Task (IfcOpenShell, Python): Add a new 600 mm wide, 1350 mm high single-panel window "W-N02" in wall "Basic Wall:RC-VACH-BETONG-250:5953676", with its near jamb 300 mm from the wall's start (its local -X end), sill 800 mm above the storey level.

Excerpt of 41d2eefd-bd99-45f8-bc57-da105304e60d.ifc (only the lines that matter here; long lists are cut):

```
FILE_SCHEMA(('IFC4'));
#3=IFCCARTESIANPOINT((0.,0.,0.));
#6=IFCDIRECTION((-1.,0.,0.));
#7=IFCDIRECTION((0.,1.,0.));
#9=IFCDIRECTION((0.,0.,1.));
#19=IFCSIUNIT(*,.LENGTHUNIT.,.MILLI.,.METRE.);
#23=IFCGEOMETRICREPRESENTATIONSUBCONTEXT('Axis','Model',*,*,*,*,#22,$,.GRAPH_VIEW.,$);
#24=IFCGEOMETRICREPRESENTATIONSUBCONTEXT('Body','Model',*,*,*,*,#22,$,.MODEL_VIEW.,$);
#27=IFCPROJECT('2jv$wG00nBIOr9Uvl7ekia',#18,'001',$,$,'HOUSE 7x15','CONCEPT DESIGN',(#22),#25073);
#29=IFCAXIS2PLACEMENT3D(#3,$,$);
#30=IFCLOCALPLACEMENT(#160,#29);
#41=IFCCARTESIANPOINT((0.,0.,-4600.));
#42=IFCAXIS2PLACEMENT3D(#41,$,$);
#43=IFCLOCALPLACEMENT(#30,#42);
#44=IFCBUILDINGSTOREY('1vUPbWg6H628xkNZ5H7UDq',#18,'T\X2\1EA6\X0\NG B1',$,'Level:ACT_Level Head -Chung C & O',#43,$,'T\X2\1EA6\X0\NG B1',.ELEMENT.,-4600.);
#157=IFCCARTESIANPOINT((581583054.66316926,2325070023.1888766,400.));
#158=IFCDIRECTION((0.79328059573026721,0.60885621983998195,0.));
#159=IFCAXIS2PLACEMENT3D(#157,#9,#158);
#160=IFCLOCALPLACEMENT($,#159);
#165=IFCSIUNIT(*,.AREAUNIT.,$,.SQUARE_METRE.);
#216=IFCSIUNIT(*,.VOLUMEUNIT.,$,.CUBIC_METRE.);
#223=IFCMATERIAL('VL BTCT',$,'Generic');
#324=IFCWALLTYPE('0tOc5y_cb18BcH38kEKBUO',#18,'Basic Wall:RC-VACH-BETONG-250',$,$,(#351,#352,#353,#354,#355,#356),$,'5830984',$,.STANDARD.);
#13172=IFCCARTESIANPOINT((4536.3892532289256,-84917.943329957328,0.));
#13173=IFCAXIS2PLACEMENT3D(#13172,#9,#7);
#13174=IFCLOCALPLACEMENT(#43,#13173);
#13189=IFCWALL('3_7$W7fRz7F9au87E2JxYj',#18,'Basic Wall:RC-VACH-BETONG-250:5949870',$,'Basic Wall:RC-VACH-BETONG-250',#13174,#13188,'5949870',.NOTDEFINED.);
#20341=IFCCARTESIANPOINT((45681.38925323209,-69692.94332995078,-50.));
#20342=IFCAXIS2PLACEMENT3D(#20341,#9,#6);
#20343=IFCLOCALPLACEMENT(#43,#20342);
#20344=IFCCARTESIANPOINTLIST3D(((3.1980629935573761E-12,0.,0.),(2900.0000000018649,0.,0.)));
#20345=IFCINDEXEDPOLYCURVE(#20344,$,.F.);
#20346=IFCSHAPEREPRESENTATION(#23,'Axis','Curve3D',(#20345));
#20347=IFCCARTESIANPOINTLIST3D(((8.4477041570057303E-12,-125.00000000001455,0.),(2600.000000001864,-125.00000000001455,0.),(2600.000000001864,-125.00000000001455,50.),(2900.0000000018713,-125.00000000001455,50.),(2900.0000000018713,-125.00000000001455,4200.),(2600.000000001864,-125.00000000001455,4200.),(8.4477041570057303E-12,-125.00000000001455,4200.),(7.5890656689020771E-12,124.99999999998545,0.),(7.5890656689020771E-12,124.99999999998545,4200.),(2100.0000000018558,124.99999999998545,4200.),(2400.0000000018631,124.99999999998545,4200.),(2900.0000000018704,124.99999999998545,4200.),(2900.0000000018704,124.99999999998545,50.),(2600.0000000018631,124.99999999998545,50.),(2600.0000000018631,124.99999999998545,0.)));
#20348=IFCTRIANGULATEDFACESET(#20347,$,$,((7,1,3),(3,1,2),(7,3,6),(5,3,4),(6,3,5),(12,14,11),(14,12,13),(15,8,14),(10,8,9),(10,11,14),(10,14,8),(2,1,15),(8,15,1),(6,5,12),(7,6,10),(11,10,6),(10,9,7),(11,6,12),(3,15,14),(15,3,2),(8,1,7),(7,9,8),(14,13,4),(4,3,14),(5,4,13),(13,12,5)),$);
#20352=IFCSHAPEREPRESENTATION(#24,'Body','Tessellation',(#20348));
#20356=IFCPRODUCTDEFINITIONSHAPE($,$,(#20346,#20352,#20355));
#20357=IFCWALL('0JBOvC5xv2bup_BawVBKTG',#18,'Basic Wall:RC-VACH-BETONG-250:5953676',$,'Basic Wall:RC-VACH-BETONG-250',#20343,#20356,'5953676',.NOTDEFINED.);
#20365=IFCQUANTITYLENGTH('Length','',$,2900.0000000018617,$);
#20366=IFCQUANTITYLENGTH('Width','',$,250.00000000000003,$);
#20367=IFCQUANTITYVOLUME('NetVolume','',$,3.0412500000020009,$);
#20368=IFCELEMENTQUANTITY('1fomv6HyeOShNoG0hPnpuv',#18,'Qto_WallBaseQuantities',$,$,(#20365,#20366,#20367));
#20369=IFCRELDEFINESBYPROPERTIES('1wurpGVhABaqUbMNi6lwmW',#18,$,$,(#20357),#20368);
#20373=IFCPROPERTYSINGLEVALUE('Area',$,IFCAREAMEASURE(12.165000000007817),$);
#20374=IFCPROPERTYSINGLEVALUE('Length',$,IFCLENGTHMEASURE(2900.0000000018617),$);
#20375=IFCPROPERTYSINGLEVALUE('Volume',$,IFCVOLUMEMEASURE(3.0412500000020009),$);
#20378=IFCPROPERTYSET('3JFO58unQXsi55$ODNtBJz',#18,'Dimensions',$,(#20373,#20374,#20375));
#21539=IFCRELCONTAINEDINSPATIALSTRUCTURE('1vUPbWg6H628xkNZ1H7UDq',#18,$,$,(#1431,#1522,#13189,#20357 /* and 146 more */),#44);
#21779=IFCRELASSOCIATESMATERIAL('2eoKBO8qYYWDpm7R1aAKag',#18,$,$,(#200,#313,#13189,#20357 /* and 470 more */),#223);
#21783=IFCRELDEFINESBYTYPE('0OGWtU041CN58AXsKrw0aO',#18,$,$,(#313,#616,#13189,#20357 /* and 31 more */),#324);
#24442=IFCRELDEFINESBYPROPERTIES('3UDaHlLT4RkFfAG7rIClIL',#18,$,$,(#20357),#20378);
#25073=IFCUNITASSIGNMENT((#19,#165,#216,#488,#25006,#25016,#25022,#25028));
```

```python
import numpy as np
import ifcopenshell
import ifcopenshell.api.feature
import ifcopenshell.api.geometry
import ifcopenshell.api.pset
import ifcopenshell.api.root
import ifcopenshell.api.spatial
import ifcopenshell.geom
import ifcopenshell.util.element
import ifcopenshell.util.placement
import ifcopenshell.util.representation
import ifcopenshell.util.shape
import ifcopenshell.util.unit

model = ifcopenshell.open("41d2eefd-bd99-45f8-bc57-da105304e60d.ifc")
unit_scale = ifcopenshell.util.unit.calculate_unit_scale(model)
area_scale = ifcopenshell.util.unit.calculate_unit_scale(model, "AREAUNIT")
volume_scale = ifcopenshell.util.unit.calculate_unit_scale(model, "VOLUMEUNIT")
settings = ifcopenshell.geom.settings()


def volume(element):
    """Net volume in cubic metres, openings subtracted."""
    shape = ifcopenshell.geom.create_shape(settings, element)
    return ifcopenshell.util.shape.get_volume(shape.geometry)


wall = model.by_guid("0JBOvC5xv2bup_BawVBKTG")
storey = ifcopenshell.util.element.get_container(wall, ifc_class="IfcBuildingStorey")
context = ifcopenshell.util.representation.get_context(model, "Model", "Body", "MODEL_VIEW")
before = volume(wall)

width, height, from_end, sill = 0.6, 1.35, 0.3, 0.8  # metres

# The wall runs along its own X axis, and the end named is its -X end.
wall_shape = ifcopenshell.geom.create_shape(settings, wall)
x, y, z = ifcopenshell.util.shape.get_vertices(wall_shape.geometry).T
start = x.min() + from_end
face, thickness = float(y.min()), float(y.max() - y.min())
wall_matrix = ifcopenshell.util.placement.get_local_placement(wall.ObjectPlacement)
level = ifcopenshell.util.placement.get_local_placement(storey.ObjectPlacement)[2, 3]


def in_wall(x, y):
    """Placement at x, y metres in the wall's axes, at sill height."""
    matrix = wall_matrix.copy()
    matrix[:, 3] = wall_matrix @ np.array([x / unit_scale, y / unit_scale, 0.0, 1.0])
    matrix[2, 3] = level + sill / unit_scale
    return matrix


# Opening: a box that overshoots both wall faces by 50 mm.
opening = ifcopenshell.api.root.create_entity(model, ifc_class="IfcOpeningElement", predefined_type="OPENING")
box = ifcopenshell.api.geometry.add_wall_representation(
    model, context=context, length=width, height=height, thickness=thickness + 0.1
)
ifcopenshell.api.geometry.assign_representation(model, product=opening, representation=box)
ifcopenshell.api.geometry.edit_object_placement(model, product=opening, matrix=in_wall(start, face - 0.05), is_si=False)
ifcopenshell.api.feature.add_feature(model, feature=opening, element=wall)

window = ifcopenshell.api.root.create_entity(model, ifc_class="IfcWindow", name="W-N02", predefined_type="WINDOW")
window.OverallWidth, window.OverallHeight = width / unit_scale, height / unit_scale
window.PartitioningType = "SINGLE_PANEL"
body = ifcopenshell.api.geometry.add_window_representation(
    model,
    context=context,
    overall_width=window.OverallWidth,
    overall_height=window.OverallHeight,
    partition_type="SINGLE_PANEL",
)
ifcopenshell.api.geometry.assign_representation(model, product=window, representation=body)
ifcopenshell.api.spatial.assign_container(model, products=[window], relating_structure=storey)
ifcopenshell.api.feature.add_filling(model, opening=opening, element=window)

# Centre the window in the wall's thickness.
ifcopenshell.api.geometry.edit_object_placement(model, product=window, matrix=in_wall(start, face), is_si=False)
window_shape = ifcopenshell.geom.create_shape(settings, window)
depth = ifcopenshell.util.shape.get_vertices(window_shape.geometry)[:, 1]
offset = face + thickness / 2 - (depth.min() + depth.max()) / 2
ifcopenshell.api.geometry.edit_object_placement(model, product=window, matrix=in_wall(start, offset), is_si=False)

after = volume(wall)

# Update the wall's stored quantities.
qto = model.by_id(ifcopenshell.util.element.get_pset(wall, "Qto_WallBaseQuantities", should_inherit=False)["id"])
ifcopenshell.api.pset.edit_qto(model, qto=qto, properties={"NetVolume": after / volume_scale})
pset = model.by_id(ifcopenshell.util.element.get_pset(wall, "Dimensions", should_inherit=False)["id"])
ifcopenshell.api.pset.edit_pset(model, pset=pset, properties={
    "Area": model.create_entity("IfcAreaMeasure", after / thickness / area_scale),
    "Volume": model.create_entity("IfcVolumeMeasure", after / volume_scale),
})

print(f"wall volume {before:.3f} -> {after:.3f} m3")

model.write("41d2eefd-bd99-45f8-bc57-da105304e60d_rev.ifc")
```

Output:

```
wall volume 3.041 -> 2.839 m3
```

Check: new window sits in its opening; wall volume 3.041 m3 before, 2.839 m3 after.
